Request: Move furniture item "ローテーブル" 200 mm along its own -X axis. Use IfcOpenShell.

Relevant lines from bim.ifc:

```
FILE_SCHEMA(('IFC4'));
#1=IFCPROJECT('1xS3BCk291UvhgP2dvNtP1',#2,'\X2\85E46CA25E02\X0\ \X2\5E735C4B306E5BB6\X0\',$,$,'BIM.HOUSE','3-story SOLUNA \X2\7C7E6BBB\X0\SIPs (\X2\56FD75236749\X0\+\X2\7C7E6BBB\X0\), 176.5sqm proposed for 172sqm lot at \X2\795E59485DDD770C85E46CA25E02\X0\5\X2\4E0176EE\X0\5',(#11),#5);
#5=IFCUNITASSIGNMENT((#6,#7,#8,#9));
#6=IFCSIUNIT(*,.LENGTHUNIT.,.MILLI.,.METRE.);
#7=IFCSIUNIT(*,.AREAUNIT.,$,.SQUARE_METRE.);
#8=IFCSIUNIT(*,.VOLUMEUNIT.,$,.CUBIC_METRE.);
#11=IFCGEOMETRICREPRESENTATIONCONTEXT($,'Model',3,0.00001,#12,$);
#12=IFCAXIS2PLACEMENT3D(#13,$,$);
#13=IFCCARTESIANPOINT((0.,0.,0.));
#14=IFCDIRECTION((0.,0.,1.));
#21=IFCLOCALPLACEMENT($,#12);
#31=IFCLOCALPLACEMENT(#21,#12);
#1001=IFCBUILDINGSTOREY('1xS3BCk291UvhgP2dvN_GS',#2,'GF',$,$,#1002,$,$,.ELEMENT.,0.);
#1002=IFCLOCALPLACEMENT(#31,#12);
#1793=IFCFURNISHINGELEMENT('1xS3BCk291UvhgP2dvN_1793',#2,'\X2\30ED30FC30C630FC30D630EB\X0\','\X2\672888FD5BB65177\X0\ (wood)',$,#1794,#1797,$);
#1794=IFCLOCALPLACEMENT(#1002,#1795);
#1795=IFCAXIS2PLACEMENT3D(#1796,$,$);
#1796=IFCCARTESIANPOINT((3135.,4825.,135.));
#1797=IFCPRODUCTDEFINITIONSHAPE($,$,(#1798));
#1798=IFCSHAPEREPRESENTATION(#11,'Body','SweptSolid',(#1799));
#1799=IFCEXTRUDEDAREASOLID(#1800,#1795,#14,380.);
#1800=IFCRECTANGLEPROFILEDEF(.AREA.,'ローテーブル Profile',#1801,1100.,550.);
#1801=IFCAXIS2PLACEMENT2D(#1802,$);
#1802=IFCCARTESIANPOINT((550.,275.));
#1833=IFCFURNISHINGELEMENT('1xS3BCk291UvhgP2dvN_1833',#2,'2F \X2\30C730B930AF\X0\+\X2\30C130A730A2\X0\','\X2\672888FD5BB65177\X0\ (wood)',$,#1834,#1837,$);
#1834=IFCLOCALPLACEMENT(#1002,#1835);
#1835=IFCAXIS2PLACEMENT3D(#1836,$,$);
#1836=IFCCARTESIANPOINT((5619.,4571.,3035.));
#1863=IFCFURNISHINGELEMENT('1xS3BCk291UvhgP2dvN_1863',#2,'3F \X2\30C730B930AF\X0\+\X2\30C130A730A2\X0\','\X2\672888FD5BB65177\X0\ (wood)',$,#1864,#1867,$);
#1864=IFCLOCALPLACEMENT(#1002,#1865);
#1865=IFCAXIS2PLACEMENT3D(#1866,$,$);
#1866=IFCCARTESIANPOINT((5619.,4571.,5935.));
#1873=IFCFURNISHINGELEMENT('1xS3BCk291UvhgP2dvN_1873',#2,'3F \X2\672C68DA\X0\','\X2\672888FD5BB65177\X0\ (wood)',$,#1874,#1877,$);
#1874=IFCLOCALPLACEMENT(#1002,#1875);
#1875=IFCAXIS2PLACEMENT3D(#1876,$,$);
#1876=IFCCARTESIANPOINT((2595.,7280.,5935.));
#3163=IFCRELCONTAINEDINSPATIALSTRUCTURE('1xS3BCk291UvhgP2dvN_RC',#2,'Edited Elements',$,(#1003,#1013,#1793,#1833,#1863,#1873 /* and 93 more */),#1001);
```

```python
import ifcopenshell
import ifcopenshell.api.geometry
import ifcopenshell.util.placement

model = ifcopenshell.open("bim.ifc")

item = model.by_guid("1xS3BCk291UvhgP2dvN_1793")
matrix = ifcopenshell.util.placement.get_local_placement(item.ObjectPlacement)
matrix[:3, 3] -= matrix[:3, 0] * 200.0
ifcopenshell.api.geometry.edit_object_placement(model, product=item, matrix=matrix, is_si=False)

print(ifcopenshell.util.placement.get_local_placement(item.ObjectPlacement).round(3) + 0.0)

model.write("bim_rev.ifc")
```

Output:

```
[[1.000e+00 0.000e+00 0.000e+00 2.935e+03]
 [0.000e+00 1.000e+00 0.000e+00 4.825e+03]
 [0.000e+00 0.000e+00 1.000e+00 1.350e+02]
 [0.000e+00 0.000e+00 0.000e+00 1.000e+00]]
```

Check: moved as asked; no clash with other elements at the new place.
